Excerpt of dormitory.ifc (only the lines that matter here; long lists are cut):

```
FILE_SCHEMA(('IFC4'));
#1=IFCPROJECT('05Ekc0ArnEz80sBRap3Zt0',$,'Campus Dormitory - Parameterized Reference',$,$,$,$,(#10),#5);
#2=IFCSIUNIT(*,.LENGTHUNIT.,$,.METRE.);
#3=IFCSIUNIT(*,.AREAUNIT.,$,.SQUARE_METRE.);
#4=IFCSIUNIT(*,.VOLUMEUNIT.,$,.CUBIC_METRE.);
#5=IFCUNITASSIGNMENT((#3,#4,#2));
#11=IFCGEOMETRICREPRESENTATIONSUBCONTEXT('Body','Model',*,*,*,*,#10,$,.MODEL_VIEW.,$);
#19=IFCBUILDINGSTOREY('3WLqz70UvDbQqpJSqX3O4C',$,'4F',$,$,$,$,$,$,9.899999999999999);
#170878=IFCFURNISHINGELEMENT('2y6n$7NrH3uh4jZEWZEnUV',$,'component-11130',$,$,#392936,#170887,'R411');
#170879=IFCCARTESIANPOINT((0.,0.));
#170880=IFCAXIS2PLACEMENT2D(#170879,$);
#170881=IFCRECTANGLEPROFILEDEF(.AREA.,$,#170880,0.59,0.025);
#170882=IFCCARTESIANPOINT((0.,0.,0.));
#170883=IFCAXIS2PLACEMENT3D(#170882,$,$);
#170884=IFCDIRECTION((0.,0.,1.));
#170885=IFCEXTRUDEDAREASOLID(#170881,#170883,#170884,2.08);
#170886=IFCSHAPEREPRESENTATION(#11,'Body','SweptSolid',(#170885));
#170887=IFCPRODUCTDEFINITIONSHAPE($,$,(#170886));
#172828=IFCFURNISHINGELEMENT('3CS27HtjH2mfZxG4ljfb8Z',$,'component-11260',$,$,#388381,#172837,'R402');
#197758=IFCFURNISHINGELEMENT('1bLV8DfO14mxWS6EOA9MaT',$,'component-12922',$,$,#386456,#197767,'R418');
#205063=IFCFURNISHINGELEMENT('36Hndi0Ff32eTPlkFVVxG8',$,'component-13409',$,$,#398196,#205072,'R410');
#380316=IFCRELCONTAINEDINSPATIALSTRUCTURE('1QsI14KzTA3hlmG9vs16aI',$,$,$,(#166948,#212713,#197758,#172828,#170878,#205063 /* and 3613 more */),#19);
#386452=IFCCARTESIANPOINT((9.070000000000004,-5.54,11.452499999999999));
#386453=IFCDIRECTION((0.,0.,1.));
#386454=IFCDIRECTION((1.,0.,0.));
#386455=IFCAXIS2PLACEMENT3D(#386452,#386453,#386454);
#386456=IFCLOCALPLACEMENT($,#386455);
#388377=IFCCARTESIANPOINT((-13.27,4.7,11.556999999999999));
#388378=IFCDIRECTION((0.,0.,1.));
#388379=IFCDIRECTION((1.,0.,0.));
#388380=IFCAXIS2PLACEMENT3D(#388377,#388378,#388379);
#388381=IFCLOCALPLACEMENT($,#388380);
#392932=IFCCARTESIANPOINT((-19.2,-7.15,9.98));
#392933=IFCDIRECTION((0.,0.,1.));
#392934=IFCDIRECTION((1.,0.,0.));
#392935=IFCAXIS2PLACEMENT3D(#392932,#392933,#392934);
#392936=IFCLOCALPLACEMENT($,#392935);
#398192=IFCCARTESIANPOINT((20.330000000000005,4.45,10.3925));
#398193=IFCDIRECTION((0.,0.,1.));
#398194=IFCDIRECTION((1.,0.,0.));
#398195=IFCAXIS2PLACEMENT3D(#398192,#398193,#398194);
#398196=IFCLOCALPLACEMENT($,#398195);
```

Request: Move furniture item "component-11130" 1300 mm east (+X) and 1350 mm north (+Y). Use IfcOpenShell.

```python
import ifcopenshell
import ifcopenshell.api.geometry
import ifcopenshell.util.placement

model = ifcopenshell.open("dormitory.ifc")

item = model.by_id(170878)
matrix = ifcopenshell.util.placement.get_local_placement(item.ObjectPlacement)
matrix[0, 3] += 1.3
matrix[1, 3] += 1.35
ifcopenshell.api.geometry.edit_object_placement(model, product=item, matrix=matrix, is_si=False)

print(ifcopenshell.util.placement.get_local_placement(item.ObjectPlacement).round(3) + 0.0)

model.write("dormitory_updated.ifc")
```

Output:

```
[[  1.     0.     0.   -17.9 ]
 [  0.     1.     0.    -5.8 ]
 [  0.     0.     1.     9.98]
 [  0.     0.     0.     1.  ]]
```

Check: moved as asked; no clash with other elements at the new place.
